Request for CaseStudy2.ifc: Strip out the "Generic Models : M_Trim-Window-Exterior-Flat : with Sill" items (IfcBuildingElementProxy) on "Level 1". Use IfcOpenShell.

First a look at what the model holds.

```python
import ifcopenshell
import ifcopenshell.util.element

model = ifcopenshell.open("CaseStudy2.ifc")
print(model.schema)
storey = next(s for s in model.by_type("IfcBuildingStorey") if s.Name == "Level 1")
proxies = [e for e in ifcopenshell.util.element.get_decomposition(storey) if e.is_a("IfcBuildingElementProxy")]
seen = {}
for e in proxies:
    element_type = ifcopenshell.util.element.get_type(e)
    name = element_type.Name if element_type not in (None, e) else None
    seen[name] = seen.get(name, 0) + 1
for name, count in sorted(seen.items(), key=str):
    print(count, "x", name)
```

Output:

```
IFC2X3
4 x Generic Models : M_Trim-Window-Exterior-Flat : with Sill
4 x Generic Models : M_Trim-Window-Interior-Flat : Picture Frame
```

```python
import ifcopenshell
import ifcopenshell.api.root
import ifcopenshell.util.element

model = ifcopenshell.open("CaseStudy2.ifc")

storey = next(s for s in model.by_type("IfcBuildingStorey") if s.Name == "Level 1")
proxies = [e for e in ifcopenshell.util.element.get_decomposition(storey) if e.is_a("IfcBuildingElementProxy")]
targets = [e for e in proxies if (t := ifcopenshell.util.element.get_type(e)) not in (None, e) and t.Name == "Generic Models : M_Trim-Window-Exterior-Flat : with Sill"]

for e in targets:
    ifcopenshell.api.root.remove_product(model, product=e)
print(len(targets), "removed")

model.write("CaseStudy2-out.ifc")
```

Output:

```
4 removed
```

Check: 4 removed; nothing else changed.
